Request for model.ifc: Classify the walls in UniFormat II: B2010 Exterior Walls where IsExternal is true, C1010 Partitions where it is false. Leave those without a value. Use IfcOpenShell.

First a look at what the model holds.

```python
import ifcopenshell
import ifcopenshell.util.element

model = ifcopenshell.open("model.ifc")
print(model.schema)
print("classifications:", [c.Name for c in model.by_type("IfcClassification")])
values = [ifcopenshell.util.element.get_pset(e, "Pset_WallCommon", "IsExternal") for e in model.by_type("IfcWall")]
for value in (True, False, None):
    print("IsExternal", value, values.count(value))
```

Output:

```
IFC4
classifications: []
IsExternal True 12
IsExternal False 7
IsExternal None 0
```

```python
import ifcopenshell
import ifcopenshell.api.classification
import ifcopenshell.util.element

model = ifcopenshell.open("model.ifc")

system = ifcopenshell.api.classification.add_classification(model, classification="UniFormat II")

walls = model.by_type("IfcWall")
external = {e: ifcopenshell.util.element.get_pset(e, "Pset_WallCommon", "IsExternal") for e in walls}
for flag, code, name in ((True, "B2010", "Exterior Walls"), (False, "C1010", "Partitions")):
    products = [e for e in walls if external[e] is flag]
    ifcopenshell.api.classification.add_reference(
        model, products=products, classification=system, identification=code, name=name
    )
    print(code, len(products))

model.write("model_rev.ifc")
```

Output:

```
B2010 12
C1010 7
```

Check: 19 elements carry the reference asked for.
